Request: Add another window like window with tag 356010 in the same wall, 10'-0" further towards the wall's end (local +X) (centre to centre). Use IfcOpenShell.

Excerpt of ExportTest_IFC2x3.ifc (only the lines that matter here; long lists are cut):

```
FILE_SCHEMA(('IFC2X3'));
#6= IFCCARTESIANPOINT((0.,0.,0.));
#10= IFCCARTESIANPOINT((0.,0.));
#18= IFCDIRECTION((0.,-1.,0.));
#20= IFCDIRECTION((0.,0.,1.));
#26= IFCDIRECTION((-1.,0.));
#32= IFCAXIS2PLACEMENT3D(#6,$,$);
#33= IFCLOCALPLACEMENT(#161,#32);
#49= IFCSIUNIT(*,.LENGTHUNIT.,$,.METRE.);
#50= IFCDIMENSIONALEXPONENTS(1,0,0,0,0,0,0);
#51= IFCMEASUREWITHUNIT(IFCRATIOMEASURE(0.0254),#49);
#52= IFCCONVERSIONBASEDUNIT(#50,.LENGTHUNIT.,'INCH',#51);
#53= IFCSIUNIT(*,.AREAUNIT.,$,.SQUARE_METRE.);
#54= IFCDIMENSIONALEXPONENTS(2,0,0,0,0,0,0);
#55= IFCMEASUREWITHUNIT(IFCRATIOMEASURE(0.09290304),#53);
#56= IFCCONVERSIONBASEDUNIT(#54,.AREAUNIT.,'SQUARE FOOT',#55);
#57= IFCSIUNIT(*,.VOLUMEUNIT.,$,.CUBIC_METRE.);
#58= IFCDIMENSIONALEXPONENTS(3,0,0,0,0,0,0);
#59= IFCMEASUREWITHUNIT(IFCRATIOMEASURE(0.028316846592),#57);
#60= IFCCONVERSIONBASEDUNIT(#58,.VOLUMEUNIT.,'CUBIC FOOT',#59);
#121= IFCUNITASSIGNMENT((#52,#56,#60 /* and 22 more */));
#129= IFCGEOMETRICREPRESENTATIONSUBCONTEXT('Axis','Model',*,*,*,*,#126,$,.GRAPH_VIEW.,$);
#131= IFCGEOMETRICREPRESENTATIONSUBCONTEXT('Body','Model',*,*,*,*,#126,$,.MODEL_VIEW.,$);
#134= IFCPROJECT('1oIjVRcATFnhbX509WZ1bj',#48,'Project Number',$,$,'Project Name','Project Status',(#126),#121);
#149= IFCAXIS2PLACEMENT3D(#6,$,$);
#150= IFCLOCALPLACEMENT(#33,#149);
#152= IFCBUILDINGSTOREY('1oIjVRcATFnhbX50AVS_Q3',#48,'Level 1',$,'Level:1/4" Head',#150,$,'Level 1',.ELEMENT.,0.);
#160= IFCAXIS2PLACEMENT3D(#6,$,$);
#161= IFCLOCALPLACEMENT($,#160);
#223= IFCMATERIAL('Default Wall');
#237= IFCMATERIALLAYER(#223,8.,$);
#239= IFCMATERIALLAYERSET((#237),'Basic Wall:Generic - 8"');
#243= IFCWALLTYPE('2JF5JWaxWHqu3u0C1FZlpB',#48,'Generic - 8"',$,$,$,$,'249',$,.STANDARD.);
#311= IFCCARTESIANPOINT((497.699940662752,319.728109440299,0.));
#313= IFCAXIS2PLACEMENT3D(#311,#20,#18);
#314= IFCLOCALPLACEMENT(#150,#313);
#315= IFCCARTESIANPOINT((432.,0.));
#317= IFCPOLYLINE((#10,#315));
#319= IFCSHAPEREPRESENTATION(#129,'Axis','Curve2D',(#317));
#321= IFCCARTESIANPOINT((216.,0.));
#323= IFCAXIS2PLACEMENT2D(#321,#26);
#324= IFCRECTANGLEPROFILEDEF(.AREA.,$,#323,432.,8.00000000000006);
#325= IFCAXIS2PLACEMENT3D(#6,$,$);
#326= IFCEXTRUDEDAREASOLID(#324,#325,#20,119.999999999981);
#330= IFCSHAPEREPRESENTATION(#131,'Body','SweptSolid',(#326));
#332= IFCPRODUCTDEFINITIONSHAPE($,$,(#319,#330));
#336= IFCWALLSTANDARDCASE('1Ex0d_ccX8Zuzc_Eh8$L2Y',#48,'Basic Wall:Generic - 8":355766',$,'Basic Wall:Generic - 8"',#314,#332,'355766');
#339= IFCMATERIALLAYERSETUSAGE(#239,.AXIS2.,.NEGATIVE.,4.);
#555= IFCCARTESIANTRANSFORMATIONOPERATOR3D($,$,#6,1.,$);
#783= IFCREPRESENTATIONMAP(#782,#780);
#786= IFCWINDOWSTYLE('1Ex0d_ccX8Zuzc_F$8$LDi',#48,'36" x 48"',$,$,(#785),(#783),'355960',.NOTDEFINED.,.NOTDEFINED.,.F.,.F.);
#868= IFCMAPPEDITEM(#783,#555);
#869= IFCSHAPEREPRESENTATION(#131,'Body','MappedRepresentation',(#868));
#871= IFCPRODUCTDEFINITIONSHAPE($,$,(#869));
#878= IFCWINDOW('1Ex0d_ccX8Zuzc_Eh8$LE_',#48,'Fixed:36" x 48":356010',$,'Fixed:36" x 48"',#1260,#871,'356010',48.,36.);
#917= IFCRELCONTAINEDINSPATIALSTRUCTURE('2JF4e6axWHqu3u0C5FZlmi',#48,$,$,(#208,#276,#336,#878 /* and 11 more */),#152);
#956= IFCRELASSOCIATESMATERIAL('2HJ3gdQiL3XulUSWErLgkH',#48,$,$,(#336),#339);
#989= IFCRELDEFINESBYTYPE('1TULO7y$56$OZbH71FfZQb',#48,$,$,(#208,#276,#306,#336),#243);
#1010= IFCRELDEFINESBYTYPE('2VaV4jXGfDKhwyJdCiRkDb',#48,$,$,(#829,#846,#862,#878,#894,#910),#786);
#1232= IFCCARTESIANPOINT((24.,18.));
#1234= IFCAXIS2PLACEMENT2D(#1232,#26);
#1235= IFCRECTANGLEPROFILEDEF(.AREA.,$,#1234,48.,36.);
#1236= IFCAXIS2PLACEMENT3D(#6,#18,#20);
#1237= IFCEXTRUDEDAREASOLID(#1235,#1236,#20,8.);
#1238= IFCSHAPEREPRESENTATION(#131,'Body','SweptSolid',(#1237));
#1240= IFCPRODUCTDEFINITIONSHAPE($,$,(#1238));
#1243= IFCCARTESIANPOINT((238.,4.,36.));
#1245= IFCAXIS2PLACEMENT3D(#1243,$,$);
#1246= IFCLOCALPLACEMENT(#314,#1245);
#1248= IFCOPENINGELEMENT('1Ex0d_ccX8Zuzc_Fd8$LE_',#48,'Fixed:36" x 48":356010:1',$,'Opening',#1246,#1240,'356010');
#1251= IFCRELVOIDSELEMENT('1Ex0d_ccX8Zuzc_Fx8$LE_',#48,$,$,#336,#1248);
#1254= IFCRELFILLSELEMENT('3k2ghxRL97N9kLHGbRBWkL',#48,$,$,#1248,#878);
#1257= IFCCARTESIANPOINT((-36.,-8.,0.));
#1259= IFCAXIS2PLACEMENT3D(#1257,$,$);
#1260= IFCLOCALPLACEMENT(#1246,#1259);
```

```python
import ifcopenshell
import ifcopenshell.api.feature
import ifcopenshell.api.geometry
import ifcopenshell.api.root
import ifcopenshell.geom
import ifcopenshell.util.element
import ifcopenshell.util.placement
import ifcopenshell.util.shape
import ifcopenshell.util.unit

model = ifcopenshell.open("ExportTest_IFC2x3.ifc")
unit_scale = ifcopenshell.util.unit.calculate_unit_scale(model)
settings = ifcopenshell.geom.settings()


def volume(element):
    """Net volume in cubic metres, openings subtracted."""
    shape = ifcopenshell.geom.create_shape(settings, element)
    return ifcopenshell.util.shape.get_volume(shape.geometry)


window = model.by_id(878)
opening = window.FillsVoids[0].RelatingOpeningElement
wall = opening.VoidsElements[0].RelatingBuildingElement
before = volume(wall)
shift = ifcopenshell.util.placement.get_local_placement(wall.ObjectPlacement)[:3, 0] * 120 * 0.0254 / unit_scale

# copy_class copies the void relationship, type, container and properties, but no geometry.
new_opening = ifcopenshell.api.root.copy_class(model, product=opening)
new_opening.Representation = ifcopenshell.util.element.copy_deep(
    model, opening.Representation, exclude=["IfcGeometricRepresentationContext", "IfcRepresentationMap"]
)
new_opening.Name = 'Fixed:36" x 48"'
new_opening.Tag = None
new_window = ifcopenshell.api.root.copy_class(model, product=window)
new_window.Representation = ifcopenshell.util.element.copy_deep(
    model, window.Representation, exclude=["IfcGeometricRepresentationContext", "IfcRepresentationMap"]
)
new_window.Name = 'Fixed:36" x 48"'
new_window.Tag = None
fills = ifcopenshell.api.feature.add_filling(model, opening=new_opening, element=new_window)
fills.OwnerHistory = new_window.OwnerHistory  # required in IFC2X3

for old, new in ((opening, new_opening), (window, new_window)):
    matrix = ifcopenshell.util.placement.get_local_placement(old.ObjectPlacement)
    matrix[:3, 3] += shift
    ifcopenshell.api.geometry.edit_object_placement(model, product=new, matrix=matrix, is_si=False)

after = volume(wall)

print(f"wall volume {before:.3f} -> {after:.3f} m3")

model.write("ExportTest_IFC2x3_rev.ifc")
```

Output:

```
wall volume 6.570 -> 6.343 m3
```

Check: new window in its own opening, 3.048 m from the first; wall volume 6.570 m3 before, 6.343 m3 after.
